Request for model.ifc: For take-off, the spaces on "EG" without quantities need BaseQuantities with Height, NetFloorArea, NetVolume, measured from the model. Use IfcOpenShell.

First a look at what the model holds.

```python
import ifcopenshell
import ifcopenshell.util.element
import ifcopenshell.util.unit

model = ifcopenshell.open("model.ifc")
print(model.schema)
for unit_type in ("LENGTHUNIT", "AREAUNIT", "VOLUMEUNIT"):
    print(unit_type, ifcopenshell.util.unit.calculate_unit_scale(model, unit_type))
storey = next(s for s in model.by_type("IfcBuildingStorey") if s.Name == "EG")
spaces = [e for e in ifcopenshell.util.element.get_decomposition(storey) if e.is_a("IfcSpace")]
for e in sorted(spaces, key=lambda e: e.id()):
    print(e.id(), e.is_a(), e.Name, list(ifcopenshell.util.element.get_psets(e, qtos_only=True)), sep=" | ")
```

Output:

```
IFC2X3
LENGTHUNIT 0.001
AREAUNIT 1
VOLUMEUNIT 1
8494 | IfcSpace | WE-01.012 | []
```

```python
import ifcopenshell
import ifcopenshell.api.pset
import ifcopenshell.geom
import ifcopenshell.util.element
import ifcopenshell.util.shape
import ifcopenshell.util.unit

model = ifcopenshell.open("model.ifc")
unit_scale = ifcopenshell.util.unit.calculate_unit_scale(model)
area_scale = ifcopenshell.util.unit.calculate_unit_scale(model, "AREAUNIT")
volume_scale = ifcopenshell.util.unit.calculate_unit_scale(model, "VOLUMEUNIT")
settings = ifcopenshell.geom.settings()

storey = next(s for s in model.by_type("IfcBuildingStorey") if s.Name == "EG")
spaces = [e for e in ifcopenshell.util.element.get_decomposition(storey) if e.is_a("IfcSpace")]

for e in sorted(spaces, key=lambda e: e.id()):
    if ifcopenshell.util.element.get_psets(e, qtos_only=True, should_inherit=False):
        continue
    # Geometry comes back in metres, in the element's own axes.
    shape = ifcopenshell.geom.create_shape(settings, e)
    values = {
        "Height": ifcopenshell.util.shape.get_z(shape.geometry) / unit_scale,
        "NetFloorArea": ifcopenshell.util.shape.get_footprint_area(shape.geometry) / area_scale,
        "NetVolume": ifcopenshell.util.shape.get_volume(shape.geometry) / volume_scale,
    }
    qto = ifcopenshell.api.pset.add_qto(model, product=e, name="BaseQuantities")
    ifcopenshell.api.pset.edit_qto(model, qto=qto, properties=values)
    print(e.id(), {k: round(v, 3) for k, v in values.items()})

model.write("model-out.ifc")
```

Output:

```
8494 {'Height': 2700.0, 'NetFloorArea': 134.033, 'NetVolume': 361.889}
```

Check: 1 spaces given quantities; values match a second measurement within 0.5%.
